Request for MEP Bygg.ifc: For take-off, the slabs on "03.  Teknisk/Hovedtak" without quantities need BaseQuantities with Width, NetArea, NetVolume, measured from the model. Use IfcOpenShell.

First a look at what the model holds.

```python
import ifcopenshell
import ifcopenshell.util.element
import ifcopenshell.util.unit

model = ifcopenshell.open("MEP Bygg.ifc")
print(model.schema)
for unit_type in ("LENGTHUNIT", "AREAUNIT", "VOLUMEUNIT"):
    print(unit_type, ifcopenshell.util.unit.calculate_unit_scale(model, unit_type))
storey = next(s for s in model.by_type("IfcBuildingStorey") if s.Name == "03.  Teknisk/Hovedtak")
slabs = [e for e in ifcopenshell.util.element.get_decomposition(storey) if e.is_a("IfcSlab")]
for e in sorted(slabs, key=lambda e: e.id()):
    print(e.id(), e.is_a(), e.Name, list(ifcopenshell.util.element.get_psets(e, qtos_only=True)), sep=" | ")
```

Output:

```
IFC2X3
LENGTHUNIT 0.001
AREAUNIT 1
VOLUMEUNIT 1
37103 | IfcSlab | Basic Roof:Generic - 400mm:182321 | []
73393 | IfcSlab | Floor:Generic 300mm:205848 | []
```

```python
import ifcopenshell
import ifcopenshell.api.pset
import ifcopenshell.geom
import ifcopenshell.util.element
import ifcopenshell.util.shape
import ifcopenshell.util.unit

model = ifcopenshell.open("MEP Bygg.ifc")
unit_scale = ifcopenshell.util.unit.calculate_unit_scale(model)
area_scale = ifcopenshell.util.unit.calculate_unit_scale(model, "AREAUNIT")
volume_scale = ifcopenshell.util.unit.calculate_unit_scale(model, "VOLUMEUNIT")
settings = ifcopenshell.geom.settings()

storey = next(s for s in model.by_type("IfcBuildingStorey") if s.Name == "03.  Teknisk/Hovedtak")
slabs = [e for e in ifcopenshell.util.element.get_decomposition(storey) if e.is_a("IfcSlab")]

for e in sorted(slabs, key=lambda e: e.id()):
    if ifcopenshell.util.element.get_psets(e, qtos_only=True, should_inherit=False):
        continue
    # Geometry comes back in metres, in the element's own axes.
    shape = ifcopenshell.geom.create_shape(settings, e)
    values = {
        "Width": ifcopenshell.util.shape.get_z(shape.geometry) / unit_scale,
        "NetArea": ifcopenshell.util.shape.get_footprint_area(shape.geometry) / area_scale,
        "NetVolume": ifcopenshell.util.shape.get_volume(shape.geometry) / volume_scale,
    }
    qto = ifcopenshell.api.pset.add_qto(model, product=e, name="BaseQuantities")
    ifcopenshell.api.pset.edit_qto(model, qto=qto, properties=values)
    print(e.id(), {k: round(v, 3) for k, v in values.items()})

model.write("MEP Bygg_v2.ifc")
```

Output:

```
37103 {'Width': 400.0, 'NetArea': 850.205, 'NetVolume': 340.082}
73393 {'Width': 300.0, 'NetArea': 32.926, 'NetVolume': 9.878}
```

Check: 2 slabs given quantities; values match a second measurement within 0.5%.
